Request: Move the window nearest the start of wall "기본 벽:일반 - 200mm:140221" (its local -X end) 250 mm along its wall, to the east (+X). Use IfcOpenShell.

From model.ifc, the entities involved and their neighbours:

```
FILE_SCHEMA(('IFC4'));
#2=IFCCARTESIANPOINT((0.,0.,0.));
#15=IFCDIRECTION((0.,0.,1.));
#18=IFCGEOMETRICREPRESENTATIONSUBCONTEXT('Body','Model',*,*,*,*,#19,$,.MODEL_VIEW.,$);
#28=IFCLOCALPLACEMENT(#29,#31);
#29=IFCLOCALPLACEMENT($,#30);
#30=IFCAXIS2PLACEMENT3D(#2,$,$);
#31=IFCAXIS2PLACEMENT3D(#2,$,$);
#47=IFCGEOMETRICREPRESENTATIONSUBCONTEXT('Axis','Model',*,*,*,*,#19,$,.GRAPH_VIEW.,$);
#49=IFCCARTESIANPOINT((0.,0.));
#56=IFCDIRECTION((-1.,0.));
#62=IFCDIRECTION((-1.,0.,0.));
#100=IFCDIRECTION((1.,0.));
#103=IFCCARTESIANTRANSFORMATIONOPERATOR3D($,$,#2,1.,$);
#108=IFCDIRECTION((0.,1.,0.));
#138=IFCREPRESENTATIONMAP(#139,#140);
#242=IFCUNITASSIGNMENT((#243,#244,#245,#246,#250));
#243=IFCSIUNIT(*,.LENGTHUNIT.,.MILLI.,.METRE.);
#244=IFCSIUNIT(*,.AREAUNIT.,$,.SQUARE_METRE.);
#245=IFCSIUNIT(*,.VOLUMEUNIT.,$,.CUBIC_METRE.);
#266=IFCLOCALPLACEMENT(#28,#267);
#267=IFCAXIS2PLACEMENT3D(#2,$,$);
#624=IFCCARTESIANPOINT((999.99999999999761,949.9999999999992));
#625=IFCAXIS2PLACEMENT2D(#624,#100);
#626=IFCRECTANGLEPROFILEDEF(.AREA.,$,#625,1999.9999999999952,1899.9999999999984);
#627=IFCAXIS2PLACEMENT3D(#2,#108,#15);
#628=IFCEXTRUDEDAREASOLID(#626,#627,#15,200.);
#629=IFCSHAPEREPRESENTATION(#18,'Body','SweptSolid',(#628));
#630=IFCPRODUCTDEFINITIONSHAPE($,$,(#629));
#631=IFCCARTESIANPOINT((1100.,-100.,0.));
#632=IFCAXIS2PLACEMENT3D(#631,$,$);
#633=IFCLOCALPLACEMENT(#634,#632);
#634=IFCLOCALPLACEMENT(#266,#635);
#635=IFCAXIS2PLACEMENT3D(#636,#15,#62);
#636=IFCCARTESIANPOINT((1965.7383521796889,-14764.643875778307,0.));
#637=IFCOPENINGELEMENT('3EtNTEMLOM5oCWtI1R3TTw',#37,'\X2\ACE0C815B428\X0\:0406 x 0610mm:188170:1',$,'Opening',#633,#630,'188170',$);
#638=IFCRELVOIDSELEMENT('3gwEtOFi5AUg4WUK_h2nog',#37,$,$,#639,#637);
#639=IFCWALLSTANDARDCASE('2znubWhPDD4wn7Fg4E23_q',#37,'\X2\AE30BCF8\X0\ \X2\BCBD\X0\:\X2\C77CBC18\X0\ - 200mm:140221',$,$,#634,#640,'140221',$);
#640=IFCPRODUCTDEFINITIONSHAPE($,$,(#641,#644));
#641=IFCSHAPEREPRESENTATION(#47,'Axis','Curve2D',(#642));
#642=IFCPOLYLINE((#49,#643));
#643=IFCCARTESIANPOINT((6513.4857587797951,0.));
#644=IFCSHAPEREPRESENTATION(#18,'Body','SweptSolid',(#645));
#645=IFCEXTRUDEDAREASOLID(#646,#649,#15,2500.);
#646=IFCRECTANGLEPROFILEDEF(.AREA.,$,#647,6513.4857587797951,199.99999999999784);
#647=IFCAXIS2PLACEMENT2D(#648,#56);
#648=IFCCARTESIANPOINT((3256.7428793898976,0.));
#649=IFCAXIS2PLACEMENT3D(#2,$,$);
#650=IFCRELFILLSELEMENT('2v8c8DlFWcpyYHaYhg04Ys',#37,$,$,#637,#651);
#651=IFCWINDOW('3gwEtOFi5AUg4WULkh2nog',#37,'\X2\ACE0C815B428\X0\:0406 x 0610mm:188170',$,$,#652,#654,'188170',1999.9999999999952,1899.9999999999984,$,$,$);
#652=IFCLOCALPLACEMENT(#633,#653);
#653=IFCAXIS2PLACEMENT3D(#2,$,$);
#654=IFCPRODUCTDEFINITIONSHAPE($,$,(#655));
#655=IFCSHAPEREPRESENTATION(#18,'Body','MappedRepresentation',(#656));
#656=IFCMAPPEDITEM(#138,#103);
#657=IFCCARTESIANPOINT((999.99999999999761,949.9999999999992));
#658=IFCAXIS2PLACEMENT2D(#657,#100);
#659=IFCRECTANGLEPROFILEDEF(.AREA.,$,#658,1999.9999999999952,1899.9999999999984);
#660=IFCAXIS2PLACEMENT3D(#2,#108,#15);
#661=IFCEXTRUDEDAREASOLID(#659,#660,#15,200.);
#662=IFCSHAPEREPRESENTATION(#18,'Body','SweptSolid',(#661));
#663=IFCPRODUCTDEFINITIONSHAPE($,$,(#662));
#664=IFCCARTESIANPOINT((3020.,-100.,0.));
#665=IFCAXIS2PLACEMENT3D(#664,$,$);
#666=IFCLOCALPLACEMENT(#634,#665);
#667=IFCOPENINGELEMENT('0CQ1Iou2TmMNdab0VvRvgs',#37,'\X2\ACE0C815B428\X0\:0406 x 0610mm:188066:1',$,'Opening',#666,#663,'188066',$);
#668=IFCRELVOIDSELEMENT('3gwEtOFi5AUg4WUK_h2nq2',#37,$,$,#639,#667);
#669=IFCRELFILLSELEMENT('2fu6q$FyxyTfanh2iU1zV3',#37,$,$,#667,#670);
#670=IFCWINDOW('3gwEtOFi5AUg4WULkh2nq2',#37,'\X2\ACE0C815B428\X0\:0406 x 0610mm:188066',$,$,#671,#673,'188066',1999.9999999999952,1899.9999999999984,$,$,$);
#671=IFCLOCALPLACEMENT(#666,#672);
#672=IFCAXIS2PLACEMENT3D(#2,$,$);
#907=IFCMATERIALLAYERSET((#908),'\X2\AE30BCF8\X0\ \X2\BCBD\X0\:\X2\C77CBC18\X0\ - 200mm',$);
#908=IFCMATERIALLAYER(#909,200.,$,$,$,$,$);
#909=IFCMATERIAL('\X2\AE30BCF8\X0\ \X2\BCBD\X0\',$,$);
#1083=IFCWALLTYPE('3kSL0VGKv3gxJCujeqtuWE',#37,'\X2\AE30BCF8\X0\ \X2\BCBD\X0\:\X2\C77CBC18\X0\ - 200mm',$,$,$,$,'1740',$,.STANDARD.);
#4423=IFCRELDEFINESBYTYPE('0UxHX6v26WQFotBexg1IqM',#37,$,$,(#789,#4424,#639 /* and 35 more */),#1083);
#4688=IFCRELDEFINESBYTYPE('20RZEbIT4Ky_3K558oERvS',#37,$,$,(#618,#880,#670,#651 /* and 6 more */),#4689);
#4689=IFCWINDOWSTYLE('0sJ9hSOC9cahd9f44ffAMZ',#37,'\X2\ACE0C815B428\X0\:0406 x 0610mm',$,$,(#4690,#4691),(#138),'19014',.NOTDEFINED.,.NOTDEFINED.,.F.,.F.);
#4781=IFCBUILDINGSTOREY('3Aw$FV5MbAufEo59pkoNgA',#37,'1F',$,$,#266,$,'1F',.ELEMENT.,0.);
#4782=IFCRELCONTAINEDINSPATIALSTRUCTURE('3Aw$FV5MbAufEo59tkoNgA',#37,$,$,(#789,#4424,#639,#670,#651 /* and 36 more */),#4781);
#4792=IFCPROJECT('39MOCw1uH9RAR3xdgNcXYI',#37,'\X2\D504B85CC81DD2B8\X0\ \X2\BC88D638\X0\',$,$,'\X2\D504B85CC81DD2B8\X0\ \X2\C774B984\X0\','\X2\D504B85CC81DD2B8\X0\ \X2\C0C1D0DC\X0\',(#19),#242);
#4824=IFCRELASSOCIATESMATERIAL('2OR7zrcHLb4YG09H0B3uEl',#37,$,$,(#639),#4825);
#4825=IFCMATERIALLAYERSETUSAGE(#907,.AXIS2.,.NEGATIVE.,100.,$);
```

```python
import ifcopenshell
import ifcopenshell.api.geometry
import ifcopenshell.util.placement

model = ifcopenshell.open("model.ifc")

window = model.by_id(651)
opening = window.FillsVoids[0].RelatingOpeningElement
wall = opening.VoidsElements[0].RelatingBuildingElement

wall_matrix = ifcopenshell.util.placement.get_local_placement(wall.ObjectPlacement)
shift = wall_matrix[:3, 0] * -250.0
before = ifcopenshell.util.placement.get_local_placement(window.ObjectPlacement)[:3, 3].copy()

# The window is placed relative to its opening, so it follows when the opening moves.
matrix = ifcopenshell.util.placement.get_local_placement(opening.ObjectPlacement)
matrix[:3, 3] += shift
ifcopenshell.api.geometry.edit_object_placement(
    model, product=opening, matrix=matrix, is_si=False, should_transform_children=True
)

after = ifcopenshell.util.placement.get_local_placement(window.ObjectPlacement)[:3, 3]
print("window moved by", (after - before).round(3) + 0.0)

model.write("model-out.ifc")
```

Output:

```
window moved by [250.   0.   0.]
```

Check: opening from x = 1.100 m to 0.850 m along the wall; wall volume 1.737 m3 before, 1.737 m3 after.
